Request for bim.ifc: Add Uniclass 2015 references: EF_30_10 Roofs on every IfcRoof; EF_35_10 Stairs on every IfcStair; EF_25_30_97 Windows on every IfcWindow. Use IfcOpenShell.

First a look at what the model holds.

```python
import ifcopenshell

model = ifcopenshell.open("bim.ifc")
print(model.schema)
print("classifications:", [c.Name for c in model.by_type("IfcClassification")])
for ifc_class in ("IfcDoor", "IfcRoof", "IfcStair", "IfcWall", "IfcWindow"):
    print(ifc_class, len(model.by_type(ifc_class)))
```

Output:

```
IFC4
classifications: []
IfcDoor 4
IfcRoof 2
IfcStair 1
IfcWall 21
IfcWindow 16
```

```python
import ifcopenshell
import ifcopenshell.api.classification

model = ifcopenshell.open("bim.ifc")

system = ifcopenshell.api.classification.add_classification(model, classification="Uniclass 2015")

codes = {
    "IfcRoof": ("EF_30_10", "Roofs"),
    "IfcStair": ("EF_35_10", "Stairs"),
    "IfcWindow": ("EF_25_30_97", "Windows"),
}
for ifc_class, (code, name) in codes.items():
    products = model.by_type(ifc_class)
    ifcopenshell.api.classification.add_reference(
        model, products=products, classification=system, identification=code, name=name
    )
    print(code, len(products))

model.write("bim_edited.ifc")
```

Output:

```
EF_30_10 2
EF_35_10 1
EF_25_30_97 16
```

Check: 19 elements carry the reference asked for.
